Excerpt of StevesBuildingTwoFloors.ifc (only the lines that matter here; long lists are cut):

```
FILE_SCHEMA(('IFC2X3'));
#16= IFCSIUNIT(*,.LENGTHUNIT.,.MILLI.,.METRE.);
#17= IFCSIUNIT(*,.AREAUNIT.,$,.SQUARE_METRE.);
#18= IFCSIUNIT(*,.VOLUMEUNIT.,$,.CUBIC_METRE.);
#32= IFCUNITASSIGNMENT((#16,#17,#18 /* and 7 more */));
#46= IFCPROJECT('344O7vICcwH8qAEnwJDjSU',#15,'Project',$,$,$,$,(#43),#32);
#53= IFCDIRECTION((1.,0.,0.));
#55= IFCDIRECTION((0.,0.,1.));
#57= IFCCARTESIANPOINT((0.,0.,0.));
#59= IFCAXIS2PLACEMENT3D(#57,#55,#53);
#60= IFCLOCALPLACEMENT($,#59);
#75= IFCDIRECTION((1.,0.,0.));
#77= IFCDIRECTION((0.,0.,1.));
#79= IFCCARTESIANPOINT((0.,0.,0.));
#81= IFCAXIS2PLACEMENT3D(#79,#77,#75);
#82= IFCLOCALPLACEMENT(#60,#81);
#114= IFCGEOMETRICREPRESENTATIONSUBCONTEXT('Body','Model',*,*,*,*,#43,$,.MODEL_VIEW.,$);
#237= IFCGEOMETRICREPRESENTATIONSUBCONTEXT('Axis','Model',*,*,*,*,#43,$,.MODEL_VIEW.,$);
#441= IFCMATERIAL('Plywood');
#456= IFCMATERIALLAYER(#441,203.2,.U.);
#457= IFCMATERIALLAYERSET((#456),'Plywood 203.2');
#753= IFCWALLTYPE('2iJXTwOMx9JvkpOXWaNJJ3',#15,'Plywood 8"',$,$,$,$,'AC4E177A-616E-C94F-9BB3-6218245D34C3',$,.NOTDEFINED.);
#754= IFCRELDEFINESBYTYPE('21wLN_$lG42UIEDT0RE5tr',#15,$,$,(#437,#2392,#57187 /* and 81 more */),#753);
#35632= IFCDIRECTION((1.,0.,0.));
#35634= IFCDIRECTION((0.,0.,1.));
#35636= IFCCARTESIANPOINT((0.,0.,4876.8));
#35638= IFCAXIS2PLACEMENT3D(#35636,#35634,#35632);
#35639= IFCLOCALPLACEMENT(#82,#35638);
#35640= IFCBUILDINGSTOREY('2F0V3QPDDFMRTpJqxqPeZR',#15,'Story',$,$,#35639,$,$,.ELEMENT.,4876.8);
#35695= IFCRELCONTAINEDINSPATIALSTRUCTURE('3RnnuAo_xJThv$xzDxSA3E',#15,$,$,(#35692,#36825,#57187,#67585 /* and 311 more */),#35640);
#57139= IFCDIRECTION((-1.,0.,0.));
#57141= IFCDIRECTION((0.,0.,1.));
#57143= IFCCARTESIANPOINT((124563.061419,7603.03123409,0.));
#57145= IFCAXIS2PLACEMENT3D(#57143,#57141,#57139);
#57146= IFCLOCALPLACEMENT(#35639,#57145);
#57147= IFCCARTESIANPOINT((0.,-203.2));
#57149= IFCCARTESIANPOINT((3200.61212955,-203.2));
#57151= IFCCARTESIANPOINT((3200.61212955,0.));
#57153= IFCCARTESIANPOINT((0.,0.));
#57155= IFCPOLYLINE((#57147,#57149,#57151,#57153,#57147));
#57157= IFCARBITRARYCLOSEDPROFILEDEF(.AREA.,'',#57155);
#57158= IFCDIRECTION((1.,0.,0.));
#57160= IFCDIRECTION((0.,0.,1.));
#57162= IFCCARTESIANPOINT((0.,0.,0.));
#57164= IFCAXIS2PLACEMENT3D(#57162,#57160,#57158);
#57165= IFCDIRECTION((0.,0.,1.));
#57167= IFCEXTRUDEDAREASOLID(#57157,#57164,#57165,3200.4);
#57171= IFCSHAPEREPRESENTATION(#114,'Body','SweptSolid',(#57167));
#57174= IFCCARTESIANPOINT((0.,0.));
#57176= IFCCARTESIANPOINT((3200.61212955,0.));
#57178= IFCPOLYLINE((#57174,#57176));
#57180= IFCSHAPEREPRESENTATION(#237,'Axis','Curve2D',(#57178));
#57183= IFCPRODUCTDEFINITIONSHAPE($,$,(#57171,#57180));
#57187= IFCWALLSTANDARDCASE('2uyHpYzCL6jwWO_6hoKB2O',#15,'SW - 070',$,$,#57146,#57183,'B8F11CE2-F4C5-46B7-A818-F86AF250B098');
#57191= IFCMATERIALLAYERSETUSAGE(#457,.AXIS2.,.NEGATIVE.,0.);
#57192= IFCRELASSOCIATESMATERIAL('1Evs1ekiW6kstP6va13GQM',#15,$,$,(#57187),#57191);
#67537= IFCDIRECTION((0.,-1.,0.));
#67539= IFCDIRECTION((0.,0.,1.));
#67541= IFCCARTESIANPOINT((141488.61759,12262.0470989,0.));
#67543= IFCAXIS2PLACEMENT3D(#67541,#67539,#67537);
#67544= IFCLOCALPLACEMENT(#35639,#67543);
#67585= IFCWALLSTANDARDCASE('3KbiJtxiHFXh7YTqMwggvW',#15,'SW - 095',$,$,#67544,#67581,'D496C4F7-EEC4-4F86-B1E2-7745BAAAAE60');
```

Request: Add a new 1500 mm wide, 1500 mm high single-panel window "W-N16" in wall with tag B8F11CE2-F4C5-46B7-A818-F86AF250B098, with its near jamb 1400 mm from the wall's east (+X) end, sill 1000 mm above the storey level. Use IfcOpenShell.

```python
import numpy as np
import ifcopenshell
import ifcopenshell.api.feature
import ifcopenshell.api.geometry
import ifcopenshell.api.root
import ifcopenshell.api.spatial
import ifcopenshell.api.type
import ifcopenshell.geom
import ifcopenshell.util.element
import ifcopenshell.util.placement
import ifcopenshell.util.representation
import ifcopenshell.util.shape
import ifcopenshell.util.unit

model = ifcopenshell.open("StevesBuildingTwoFloors.ifc")
unit_scale = ifcopenshell.util.unit.calculate_unit_scale(model)
settings = ifcopenshell.geom.settings()


def volume(element):
    """Net volume in cubic metres, openings subtracted."""
    shape = ifcopenshell.geom.create_shape(settings, element)
    return ifcopenshell.util.shape.get_volume(shape.geometry)


wall = model.by_guid("2uyHpYzCL6jwWO_6hoKB2O")
storey = ifcopenshell.util.element.get_container(wall, ifc_class="IfcBuildingStorey")
context = ifcopenshell.util.representation.get_context(model, "Model", "Body", "MODEL_VIEW")
before = volume(wall)

width, height, from_end, sill = 1.5, 1.5, 1.4, 1  # metres

# The wall runs along its own X axis, and the end named is its -X end.
wall_shape = ifcopenshell.geom.create_shape(settings, wall)
x, y, z = ifcopenshell.util.shape.get_vertices(wall_shape.geometry).T
start = x.min() + from_end
face, thickness = float(y.min()), float(y.max() - y.min())
wall_matrix = ifcopenshell.util.placement.get_local_placement(wall.ObjectPlacement)
level = ifcopenshell.util.placement.get_local_placement(storey.ObjectPlacement)[2, 3]


def in_wall(x, y):
    """Placement at x, y metres in the wall's axes, at sill height."""
    matrix = wall_matrix.copy()
    matrix[:, 3] = wall_matrix @ np.array([x / unit_scale, y / unit_scale, 0.0, 1.0])
    matrix[2, 3] = level + sill / unit_scale
    return matrix


# Opening: a box that overshoots both wall faces by 50 mm.
opening = ifcopenshell.api.root.create_entity(model, ifc_class="IfcOpeningElement")
box = ifcopenshell.api.geometry.add_wall_representation(
    model, context=context, length=width, height=height, thickness=thickness + 0.1
)
ifcopenshell.api.geometry.assign_representation(model, product=opening, representation=box)
ifcopenshell.api.geometry.edit_object_placement(model, product=opening, matrix=in_wall(start, face - 0.05), is_si=False)
ifcopenshell.api.feature.add_feature(model, feature=opening, element=wall)

window = ifcopenshell.api.root.create_entity(model, ifc_class="IfcWindow", name="W-N16")
window.OverallWidth, window.OverallHeight = width / unit_scale, height / unit_scale
body = ifcopenshell.api.geometry.add_window_representation(
    model,
    context=context,
    overall_width=window.OverallWidth,
    overall_height=window.OverallHeight,
    partition_type="SINGLE_PANEL",
)
ifcopenshell.api.geometry.assign_representation(model, product=window, representation=body)
ifcopenshell.api.spatial.assign_container(model, products=[window], relating_structure=storey)
fills = ifcopenshell.api.feature.add_filling(model, opening=opening, element=window)
fills.OwnerHistory = window.OwnerHistory  # required in IFC2X3

# IFC2X3 keeps the operation on the window style.
style = ifcopenshell.api.root.create_entity(model, ifc_class="IfcWindowStyle", name="W-N16")
style.OperationType, style.ConstructionType = "SINGLE_PANEL", "NOTDEFINED"
style.ParameterTakesPrecedence = style.Sizeable = False
ifcopenshell.api.type.assign_type(model, related_objects=[window], relating_type=style)

# Centre the window in the wall's thickness.
ifcopenshell.api.geometry.edit_object_placement(model, product=window, matrix=in_wall(start, face), is_si=False)
window_shape = ifcopenshell.geom.create_shape(settings, window)
depth = ifcopenshell.util.shape.get_vertices(window_shape.geometry)[:, 1]
offset = face + thickness / 2 - (depth.min() + depth.max()) / 2
ifcopenshell.api.geometry.edit_object_placement(model, product=window, matrix=in_wall(start, offset), is_si=False)

after = volume(wall)

print(f"wall volume {before:.3f} -> {after:.3f} m3")

model.write("StevesBuildingTwoFloors_rev.ifc")
```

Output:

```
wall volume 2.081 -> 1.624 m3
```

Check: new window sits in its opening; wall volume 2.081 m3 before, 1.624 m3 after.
